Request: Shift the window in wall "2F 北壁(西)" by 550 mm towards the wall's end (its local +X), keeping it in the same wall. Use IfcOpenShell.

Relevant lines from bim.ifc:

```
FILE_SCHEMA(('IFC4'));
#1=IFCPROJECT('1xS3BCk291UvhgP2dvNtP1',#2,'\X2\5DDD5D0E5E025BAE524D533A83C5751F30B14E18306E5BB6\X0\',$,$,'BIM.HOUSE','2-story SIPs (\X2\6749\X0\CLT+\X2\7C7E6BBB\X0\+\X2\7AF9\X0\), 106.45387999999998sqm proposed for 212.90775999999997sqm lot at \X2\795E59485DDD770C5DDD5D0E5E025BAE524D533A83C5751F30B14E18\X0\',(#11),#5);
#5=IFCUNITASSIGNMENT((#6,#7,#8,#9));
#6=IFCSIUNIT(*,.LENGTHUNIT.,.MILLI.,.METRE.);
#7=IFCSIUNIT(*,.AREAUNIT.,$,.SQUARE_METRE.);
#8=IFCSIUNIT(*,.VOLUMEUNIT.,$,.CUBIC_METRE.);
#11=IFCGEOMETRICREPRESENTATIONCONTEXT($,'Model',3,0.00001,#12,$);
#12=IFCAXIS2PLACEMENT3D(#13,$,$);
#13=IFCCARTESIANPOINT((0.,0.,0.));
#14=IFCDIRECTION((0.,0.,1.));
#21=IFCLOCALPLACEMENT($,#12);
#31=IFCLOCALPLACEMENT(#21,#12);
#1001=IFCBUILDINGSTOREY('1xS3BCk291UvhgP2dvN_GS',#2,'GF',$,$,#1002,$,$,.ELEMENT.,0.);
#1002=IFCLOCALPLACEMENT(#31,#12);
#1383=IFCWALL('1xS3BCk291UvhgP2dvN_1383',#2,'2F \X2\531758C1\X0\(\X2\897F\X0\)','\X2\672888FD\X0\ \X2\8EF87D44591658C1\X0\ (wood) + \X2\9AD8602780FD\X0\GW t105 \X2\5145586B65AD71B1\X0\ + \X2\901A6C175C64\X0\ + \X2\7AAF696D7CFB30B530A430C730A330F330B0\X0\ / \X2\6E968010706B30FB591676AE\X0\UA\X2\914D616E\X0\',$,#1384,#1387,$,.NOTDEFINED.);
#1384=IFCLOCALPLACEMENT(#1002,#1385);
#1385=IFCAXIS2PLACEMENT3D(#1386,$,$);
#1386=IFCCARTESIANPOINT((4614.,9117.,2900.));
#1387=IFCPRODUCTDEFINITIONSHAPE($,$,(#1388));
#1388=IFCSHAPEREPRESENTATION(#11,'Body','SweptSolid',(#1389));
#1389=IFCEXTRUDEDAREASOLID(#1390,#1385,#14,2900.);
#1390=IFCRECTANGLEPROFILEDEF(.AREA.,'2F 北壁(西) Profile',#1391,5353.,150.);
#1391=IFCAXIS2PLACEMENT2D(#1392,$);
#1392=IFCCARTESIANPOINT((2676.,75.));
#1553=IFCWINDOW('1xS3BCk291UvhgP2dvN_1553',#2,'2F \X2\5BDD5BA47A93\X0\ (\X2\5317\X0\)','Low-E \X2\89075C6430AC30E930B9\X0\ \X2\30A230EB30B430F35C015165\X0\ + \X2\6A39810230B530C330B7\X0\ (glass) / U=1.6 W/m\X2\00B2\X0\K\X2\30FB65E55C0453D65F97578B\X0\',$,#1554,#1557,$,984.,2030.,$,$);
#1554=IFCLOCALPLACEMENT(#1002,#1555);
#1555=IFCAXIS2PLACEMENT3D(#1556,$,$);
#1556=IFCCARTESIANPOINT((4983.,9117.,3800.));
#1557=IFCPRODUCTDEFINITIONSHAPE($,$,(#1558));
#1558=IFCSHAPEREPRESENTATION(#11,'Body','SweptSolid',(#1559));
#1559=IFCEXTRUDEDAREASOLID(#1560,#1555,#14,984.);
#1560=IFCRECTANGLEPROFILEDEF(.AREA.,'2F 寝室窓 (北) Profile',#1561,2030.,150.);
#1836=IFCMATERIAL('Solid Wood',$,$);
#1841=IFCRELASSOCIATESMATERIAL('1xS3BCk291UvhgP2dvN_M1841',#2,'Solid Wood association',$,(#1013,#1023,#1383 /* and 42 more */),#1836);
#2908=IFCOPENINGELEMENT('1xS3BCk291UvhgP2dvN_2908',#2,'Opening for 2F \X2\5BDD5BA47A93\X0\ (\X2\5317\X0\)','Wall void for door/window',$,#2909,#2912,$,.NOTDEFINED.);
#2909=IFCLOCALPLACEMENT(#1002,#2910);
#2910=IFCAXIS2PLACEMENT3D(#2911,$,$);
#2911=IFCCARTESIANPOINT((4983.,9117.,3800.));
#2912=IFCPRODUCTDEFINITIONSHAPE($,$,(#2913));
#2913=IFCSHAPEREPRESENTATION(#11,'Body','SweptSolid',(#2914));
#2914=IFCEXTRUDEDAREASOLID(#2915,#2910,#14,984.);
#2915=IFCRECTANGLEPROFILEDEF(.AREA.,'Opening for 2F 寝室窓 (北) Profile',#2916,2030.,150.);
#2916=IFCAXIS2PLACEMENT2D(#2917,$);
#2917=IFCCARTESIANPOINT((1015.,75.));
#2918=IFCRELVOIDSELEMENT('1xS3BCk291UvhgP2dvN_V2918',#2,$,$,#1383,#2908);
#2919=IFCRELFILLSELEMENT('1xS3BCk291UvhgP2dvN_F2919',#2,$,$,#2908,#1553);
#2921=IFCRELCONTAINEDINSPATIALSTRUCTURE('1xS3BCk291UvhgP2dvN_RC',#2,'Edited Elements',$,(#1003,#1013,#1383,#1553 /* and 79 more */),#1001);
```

```python
import ifcopenshell
import ifcopenshell.api.geometry
import ifcopenshell.util.placement

model = ifcopenshell.open("bim.ifc")

window = model.by_guid("1xS3BCk291UvhgP2dvN_1553")
opening = window.FillsVoids[0].RelatingOpeningElement
wall = opening.VoidsElements[0].RelatingBuildingElement

wall_matrix = ifcopenshell.util.placement.get_local_placement(wall.ObjectPlacement)
shift = wall_matrix[:3, 0] * 550.0
before = ifcopenshell.util.placement.get_local_placement(window.ObjectPlacement)[:3, 3].copy()

# The window is not placed relative to its opening, so move both.
for product in (opening, window):
    matrix = ifcopenshell.util.placement.get_local_placement(product.ObjectPlacement)
    matrix[:3, 3] += shift
    ifcopenshell.api.geometry.edit_object_placement(model, product=product, matrix=matrix, is_si=False)

after = ifcopenshell.util.placement.get_local_placement(window.ObjectPlacement)[:3, 3]
print("window moved by", (after - before).round(3) + 0.0)

model.write("bim_updated.ifc")
```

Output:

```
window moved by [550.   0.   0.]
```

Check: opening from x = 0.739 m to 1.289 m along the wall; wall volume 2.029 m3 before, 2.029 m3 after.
